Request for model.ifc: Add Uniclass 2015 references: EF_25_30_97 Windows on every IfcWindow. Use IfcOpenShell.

First a look at what the model holds.

```python
import ifcopenshell

model = ifcopenshell.open("model.ifc")
print(model.schema)
print("classifications:", [c.Name for c in model.by_type("IfcClassification")])
for ifc_class in ("IfcDoor", "IfcRoof", "IfcStair", "IfcWall", "IfcWindow"):
    print(ifc_class, len(model.by_type(ifc_class)))
```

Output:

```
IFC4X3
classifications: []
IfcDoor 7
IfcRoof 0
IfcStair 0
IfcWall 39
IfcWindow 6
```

```python
import ifcopenshell
import ifcopenshell.api.classification

model = ifcopenshell.open("model.ifc")

system = ifcopenshell.api.classification.add_classification(model, classification="Uniclass 2015")

codes = {
    "IfcWindow": ("EF_25_30_97", "Windows"),
}
for ifc_class, (code, name) in codes.items():
    products = model.by_type(ifc_class)
    ifcopenshell.api.classification.add_reference(
        model, products=products, classification=system, identification=code, name=name
    )
    print(code, len(products))

model.write("model_rev.ifc")
```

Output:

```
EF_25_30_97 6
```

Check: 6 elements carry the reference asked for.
